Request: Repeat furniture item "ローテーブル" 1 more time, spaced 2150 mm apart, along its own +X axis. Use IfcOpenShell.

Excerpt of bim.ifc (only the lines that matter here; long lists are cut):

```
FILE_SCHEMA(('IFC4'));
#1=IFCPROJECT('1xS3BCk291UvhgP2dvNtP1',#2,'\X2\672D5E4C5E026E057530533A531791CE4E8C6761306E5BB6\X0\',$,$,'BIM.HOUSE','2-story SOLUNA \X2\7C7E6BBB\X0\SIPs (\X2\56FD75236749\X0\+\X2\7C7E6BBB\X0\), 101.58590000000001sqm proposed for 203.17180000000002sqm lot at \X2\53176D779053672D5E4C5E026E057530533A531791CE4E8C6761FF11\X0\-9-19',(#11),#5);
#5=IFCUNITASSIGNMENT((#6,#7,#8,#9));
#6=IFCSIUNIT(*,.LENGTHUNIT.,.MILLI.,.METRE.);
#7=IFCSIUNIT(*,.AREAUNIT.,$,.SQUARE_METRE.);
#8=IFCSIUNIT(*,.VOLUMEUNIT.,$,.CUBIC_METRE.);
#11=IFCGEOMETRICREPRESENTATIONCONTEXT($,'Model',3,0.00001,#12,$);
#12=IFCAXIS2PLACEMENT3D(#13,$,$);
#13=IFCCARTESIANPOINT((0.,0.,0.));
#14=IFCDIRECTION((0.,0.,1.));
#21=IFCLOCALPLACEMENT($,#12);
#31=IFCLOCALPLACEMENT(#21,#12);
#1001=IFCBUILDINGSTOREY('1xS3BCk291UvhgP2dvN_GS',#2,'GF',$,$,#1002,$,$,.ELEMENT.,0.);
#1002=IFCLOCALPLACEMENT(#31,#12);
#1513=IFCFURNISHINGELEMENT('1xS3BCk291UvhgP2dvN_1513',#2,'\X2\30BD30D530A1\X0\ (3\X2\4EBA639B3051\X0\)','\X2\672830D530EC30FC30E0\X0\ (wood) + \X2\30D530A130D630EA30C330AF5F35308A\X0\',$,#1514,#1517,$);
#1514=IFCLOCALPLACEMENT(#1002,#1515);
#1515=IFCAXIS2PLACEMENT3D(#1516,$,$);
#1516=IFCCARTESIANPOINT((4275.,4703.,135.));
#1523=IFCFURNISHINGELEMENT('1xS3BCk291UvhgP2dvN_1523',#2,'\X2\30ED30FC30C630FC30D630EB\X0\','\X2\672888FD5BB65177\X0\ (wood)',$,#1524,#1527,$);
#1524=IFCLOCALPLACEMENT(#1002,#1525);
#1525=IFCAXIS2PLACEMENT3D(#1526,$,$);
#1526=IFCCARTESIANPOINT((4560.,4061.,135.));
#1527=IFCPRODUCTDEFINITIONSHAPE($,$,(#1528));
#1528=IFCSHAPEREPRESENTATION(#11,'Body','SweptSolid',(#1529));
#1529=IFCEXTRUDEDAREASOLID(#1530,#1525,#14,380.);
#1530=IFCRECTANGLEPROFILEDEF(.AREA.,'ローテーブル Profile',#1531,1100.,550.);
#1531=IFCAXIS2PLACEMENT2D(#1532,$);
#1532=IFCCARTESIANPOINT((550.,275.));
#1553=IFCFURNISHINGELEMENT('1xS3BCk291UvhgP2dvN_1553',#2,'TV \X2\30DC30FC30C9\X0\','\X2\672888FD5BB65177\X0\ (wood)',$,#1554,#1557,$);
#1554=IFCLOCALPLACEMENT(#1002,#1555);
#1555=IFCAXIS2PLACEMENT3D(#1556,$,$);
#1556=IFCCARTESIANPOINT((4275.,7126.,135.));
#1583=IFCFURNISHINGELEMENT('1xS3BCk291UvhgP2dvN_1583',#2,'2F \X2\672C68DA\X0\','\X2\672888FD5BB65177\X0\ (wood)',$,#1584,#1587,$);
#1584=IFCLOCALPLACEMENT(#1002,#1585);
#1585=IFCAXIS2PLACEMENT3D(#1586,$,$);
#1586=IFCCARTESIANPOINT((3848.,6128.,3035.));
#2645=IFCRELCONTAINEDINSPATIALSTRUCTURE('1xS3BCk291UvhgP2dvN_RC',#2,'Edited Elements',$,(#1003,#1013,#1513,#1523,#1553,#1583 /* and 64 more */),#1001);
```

```python
import ifcopenshell
import ifcopenshell.api.geometry
import ifcopenshell.api.root
import ifcopenshell.util.element
import ifcopenshell.util.placement
import ifcopenshell.util.unit

model = ifcopenshell.open("bim.ifc")
unit_scale = ifcopenshell.util.unit.calculate_unit_scale(model)


def reuse_history(source, copy):
    """copy_class also copies each property set's owner history, people and application; keep the originals."""
    for rel in copy.IsDefinedBy:
        if rel.is_a("IfcRelDefinesByProperties") and (history := rel.RelatingPropertyDefinition.OwnerHistory):
            rel.RelatingPropertyDefinition.OwnerHistory = source.OwnerHistory
            ifcopenshell.util.element.remove_deep2(model, history)


source = model.by_guid("1xS3BCk291UvhgP2dvN_1523")
base = ifcopenshell.util.placement.get_local_placement(source.ObjectPlacement)
step = base[:3, 0] * 2.15 / unit_scale

for i in range(1, 2):
    copy = ifcopenshell.api.root.copy_class(model, product=source)
    copy.Representation = ifcopenshell.util.element.copy_deep(
        model, source.Representation, exclude=["IfcGeometricRepresentationContext", "IfcRepresentationMap"]
    )
    reuse_history(source, copy)
    matrix = base.copy()
    matrix[:3, 3] += i * step
    print("added at", matrix[:3, 3].round(3) + 0.0)
    ifcopenshell.api.geometry.edit_object_placement(model, product=copy, matrix=matrix, is_si=False)

model.write("bim-out.ifc")
```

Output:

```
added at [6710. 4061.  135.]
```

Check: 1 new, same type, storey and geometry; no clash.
